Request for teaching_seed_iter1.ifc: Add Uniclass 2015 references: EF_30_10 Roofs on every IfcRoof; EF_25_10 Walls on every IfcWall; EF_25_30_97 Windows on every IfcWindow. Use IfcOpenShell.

First a look at what the model holds.

```python
import ifcopenshell

model = ifcopenshell.open("teaching_seed_iter1.ifc")
print(model.schema)
print("classifications:", [c.Name for c in model.by_type("IfcClassification")])
for ifc_class in ("IfcDoor", "IfcRoof", "IfcStair", "IfcWall", "IfcWindow"):
    print(ifc_class, len(model.by_type(ifc_class)))
```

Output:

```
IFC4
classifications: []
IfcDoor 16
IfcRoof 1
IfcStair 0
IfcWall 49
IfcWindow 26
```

```python
import ifcopenshell
import ifcopenshell.api.classification

model = ifcopenshell.open("teaching_seed_iter1.ifc")

system = ifcopenshell.api.classification.add_classification(model, classification="Uniclass 2015")

codes = {
    "IfcRoof": ("EF_30_10", "Roofs"),
    "IfcWall": ("EF_25_10", "Walls"),
    "IfcWindow": ("EF_25_30_97", "Windows"),
}
for ifc_class, (code, name) in codes.items():
    products = model.by_type(ifc_class)
    ifcopenshell.api.classification.add_reference(
        model, products=products, classification=system, identification=code, name=name
    )
    print(code, len(products))

model.write("teaching_seed_iter1_rev.ifc")
```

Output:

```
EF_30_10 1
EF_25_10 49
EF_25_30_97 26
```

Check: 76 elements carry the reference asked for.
